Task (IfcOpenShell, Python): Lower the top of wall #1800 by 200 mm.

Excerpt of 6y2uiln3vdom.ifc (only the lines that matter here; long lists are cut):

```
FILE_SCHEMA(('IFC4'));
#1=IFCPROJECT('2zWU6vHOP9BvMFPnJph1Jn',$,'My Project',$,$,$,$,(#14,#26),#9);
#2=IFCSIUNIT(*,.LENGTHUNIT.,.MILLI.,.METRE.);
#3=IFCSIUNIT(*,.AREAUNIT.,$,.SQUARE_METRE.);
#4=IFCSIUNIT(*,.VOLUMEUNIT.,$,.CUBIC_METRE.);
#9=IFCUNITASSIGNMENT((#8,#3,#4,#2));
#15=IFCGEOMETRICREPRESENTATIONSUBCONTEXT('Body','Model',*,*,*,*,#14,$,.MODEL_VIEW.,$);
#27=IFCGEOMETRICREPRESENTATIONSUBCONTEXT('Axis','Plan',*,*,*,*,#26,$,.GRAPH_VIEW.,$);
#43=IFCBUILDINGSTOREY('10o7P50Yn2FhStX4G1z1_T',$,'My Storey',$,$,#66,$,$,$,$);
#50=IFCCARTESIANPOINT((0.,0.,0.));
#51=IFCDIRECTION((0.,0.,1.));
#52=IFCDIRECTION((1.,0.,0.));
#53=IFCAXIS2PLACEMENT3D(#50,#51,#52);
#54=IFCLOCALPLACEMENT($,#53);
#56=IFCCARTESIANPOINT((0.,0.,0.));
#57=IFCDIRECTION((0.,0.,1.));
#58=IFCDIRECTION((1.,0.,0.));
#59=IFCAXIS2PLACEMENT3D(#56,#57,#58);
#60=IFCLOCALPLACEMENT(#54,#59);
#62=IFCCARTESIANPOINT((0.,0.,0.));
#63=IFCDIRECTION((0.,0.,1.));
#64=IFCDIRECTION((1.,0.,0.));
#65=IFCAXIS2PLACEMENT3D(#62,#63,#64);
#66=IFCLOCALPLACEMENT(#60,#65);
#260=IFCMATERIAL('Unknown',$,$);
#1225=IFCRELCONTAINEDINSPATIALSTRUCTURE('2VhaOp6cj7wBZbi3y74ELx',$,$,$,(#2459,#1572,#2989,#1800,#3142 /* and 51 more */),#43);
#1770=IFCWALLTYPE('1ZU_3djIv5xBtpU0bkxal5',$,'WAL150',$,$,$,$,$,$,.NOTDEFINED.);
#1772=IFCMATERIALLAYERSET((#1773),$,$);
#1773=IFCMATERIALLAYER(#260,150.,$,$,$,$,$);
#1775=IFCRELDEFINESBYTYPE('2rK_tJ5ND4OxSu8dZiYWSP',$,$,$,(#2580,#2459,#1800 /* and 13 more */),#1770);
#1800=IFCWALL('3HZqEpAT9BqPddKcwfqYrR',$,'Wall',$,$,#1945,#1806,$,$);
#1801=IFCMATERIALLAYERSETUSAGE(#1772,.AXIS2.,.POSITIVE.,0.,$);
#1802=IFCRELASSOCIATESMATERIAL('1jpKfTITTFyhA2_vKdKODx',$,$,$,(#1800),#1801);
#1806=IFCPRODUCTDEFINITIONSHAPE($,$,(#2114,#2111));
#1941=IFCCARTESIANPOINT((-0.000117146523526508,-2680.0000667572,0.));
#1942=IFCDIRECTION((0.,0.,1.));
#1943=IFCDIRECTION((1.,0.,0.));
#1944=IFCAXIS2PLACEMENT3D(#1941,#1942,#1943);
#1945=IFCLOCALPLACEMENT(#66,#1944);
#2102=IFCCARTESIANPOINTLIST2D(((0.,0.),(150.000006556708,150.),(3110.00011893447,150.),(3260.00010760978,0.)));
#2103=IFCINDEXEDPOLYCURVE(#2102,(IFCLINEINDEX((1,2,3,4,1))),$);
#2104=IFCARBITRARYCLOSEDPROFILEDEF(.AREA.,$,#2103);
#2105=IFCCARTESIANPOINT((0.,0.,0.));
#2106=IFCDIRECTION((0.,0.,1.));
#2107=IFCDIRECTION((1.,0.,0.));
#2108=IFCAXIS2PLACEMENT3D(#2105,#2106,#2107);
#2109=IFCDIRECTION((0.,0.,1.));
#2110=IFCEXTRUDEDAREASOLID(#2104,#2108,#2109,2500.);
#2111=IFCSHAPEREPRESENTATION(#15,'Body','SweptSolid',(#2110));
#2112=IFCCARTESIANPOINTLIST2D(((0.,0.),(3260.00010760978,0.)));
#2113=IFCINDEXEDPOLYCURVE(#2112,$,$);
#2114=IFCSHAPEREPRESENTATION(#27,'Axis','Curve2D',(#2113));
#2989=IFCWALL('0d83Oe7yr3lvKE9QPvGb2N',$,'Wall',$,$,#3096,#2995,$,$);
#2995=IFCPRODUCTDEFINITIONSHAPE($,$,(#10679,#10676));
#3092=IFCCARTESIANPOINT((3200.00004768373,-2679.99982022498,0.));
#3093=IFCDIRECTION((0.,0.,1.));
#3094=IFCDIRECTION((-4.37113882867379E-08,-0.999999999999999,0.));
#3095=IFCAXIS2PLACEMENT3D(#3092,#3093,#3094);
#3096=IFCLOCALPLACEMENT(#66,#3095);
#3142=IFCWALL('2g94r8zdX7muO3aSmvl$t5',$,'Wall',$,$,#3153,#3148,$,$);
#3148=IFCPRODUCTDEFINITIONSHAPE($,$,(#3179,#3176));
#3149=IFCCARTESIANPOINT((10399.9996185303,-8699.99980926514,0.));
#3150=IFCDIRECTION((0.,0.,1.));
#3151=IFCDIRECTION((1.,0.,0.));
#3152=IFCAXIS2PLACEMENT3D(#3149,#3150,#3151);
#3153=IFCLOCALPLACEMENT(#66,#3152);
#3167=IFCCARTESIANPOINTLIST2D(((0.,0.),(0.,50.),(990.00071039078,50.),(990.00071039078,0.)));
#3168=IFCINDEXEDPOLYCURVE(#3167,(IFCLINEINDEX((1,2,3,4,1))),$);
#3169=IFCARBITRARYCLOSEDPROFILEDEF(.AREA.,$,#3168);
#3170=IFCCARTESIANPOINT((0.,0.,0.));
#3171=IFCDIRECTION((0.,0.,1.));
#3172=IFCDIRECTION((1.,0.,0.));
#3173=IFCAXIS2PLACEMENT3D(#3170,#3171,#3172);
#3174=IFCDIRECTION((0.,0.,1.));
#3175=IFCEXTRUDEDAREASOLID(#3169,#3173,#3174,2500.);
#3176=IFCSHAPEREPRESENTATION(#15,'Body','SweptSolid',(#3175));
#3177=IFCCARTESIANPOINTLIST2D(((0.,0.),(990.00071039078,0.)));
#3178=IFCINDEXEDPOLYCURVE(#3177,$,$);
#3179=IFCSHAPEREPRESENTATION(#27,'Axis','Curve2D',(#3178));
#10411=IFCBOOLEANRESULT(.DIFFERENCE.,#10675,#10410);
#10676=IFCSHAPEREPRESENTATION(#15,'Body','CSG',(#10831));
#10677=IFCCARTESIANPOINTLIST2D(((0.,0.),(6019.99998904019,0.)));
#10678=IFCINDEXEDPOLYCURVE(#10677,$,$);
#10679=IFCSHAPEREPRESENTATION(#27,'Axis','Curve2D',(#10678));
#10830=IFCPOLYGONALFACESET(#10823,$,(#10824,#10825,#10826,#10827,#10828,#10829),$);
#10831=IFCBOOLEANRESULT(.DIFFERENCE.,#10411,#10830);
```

```python
import ifcopenshell
import ifcopenshell.geom
import ifcopenshell.util.representation
import ifcopenshell.util.shape

model = ifcopenshell.open("6y2uiln3vdom.ifc")
settings = ifcopenshell.geom.settings()


def volume(element):
    """Net volume in cubic metres, openings subtracted."""
    shape = ifcopenshell.geom.create_shape(settings, element)
    return ifcopenshell.util.shape.get_volume(shape.geometry)


wall = model.by_guid("3HZqEpAT9BqPddKcwfqYrR")
before = volume(wall)

body = ifcopenshell.util.representation.get_representation(wall, "Model", "Body")
solid = body.Items[0]
old_height = solid.Depth
solid.Depth -= 200.0
after = volume(wall)

print(f"height {old_height:g} -> {solid.Depth:g}, volume {before:.3f} -> {after:.3f} m3")

model.write("6y2uiln3vdom-out.ifc")
```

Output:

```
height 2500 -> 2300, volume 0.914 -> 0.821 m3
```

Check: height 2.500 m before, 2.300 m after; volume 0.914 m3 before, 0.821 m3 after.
